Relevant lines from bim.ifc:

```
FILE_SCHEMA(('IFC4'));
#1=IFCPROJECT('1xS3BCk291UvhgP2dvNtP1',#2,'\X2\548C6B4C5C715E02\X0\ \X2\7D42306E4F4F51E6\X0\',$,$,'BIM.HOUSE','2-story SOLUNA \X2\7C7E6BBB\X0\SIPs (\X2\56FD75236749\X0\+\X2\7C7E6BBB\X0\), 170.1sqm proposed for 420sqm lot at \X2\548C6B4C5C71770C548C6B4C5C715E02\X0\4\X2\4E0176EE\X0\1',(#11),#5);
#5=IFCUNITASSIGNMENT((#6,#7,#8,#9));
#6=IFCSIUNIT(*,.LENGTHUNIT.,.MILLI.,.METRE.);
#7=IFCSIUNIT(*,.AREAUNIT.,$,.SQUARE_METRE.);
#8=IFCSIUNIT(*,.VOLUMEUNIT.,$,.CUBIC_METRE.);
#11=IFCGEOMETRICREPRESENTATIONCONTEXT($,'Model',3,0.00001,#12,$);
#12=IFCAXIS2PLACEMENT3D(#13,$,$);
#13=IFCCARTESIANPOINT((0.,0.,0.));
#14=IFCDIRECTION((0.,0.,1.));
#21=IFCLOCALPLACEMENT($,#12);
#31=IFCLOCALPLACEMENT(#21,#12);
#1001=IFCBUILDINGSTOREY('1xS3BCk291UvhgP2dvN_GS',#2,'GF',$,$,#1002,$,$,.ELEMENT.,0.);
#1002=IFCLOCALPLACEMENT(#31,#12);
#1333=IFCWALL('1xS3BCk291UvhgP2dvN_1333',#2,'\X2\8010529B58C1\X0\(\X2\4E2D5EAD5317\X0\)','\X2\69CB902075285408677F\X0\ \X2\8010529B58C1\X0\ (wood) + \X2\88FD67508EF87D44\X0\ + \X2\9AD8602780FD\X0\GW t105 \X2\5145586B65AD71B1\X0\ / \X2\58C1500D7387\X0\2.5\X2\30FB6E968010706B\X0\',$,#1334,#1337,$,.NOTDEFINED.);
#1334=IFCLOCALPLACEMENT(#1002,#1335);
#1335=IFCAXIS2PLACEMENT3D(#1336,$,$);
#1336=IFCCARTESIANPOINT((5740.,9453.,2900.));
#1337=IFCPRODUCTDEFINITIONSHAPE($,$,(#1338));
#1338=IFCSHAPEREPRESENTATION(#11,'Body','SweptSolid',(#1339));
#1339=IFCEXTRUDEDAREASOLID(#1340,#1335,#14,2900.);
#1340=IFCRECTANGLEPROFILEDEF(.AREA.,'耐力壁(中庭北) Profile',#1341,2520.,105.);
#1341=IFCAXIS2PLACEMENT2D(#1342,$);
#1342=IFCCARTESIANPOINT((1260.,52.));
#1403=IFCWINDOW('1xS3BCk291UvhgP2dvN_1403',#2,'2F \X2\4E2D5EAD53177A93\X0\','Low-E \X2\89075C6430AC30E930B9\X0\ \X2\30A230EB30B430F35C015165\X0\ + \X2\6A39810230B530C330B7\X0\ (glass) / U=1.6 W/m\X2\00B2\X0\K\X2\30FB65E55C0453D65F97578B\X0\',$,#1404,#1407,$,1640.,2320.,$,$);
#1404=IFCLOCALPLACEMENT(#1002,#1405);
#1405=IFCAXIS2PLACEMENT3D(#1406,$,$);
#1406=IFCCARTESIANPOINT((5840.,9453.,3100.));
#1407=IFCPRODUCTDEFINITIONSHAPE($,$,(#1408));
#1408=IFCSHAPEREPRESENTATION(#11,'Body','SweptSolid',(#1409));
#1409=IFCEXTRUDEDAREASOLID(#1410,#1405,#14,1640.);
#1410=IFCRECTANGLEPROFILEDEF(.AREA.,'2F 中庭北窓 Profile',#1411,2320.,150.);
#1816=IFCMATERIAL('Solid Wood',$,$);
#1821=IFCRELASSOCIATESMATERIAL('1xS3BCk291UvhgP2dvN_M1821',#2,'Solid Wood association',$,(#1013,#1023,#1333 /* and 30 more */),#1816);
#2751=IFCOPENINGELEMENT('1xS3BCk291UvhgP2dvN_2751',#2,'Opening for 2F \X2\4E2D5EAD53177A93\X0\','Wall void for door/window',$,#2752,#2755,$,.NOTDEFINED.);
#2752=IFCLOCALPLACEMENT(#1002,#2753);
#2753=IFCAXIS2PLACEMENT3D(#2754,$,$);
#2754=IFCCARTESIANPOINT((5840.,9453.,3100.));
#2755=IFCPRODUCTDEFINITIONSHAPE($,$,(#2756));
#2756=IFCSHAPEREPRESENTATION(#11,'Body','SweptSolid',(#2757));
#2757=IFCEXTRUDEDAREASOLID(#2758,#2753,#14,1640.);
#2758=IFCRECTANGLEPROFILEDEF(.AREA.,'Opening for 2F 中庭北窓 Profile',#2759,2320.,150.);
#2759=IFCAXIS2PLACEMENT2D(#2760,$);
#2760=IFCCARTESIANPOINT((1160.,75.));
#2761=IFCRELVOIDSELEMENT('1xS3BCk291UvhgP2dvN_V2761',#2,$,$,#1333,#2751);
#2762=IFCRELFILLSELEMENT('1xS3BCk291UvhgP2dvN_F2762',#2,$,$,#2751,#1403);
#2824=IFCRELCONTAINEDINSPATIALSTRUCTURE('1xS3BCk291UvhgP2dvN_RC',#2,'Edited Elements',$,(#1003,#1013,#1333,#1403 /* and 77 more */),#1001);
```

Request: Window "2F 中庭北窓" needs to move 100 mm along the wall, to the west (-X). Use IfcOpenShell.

```python
import ifcopenshell
import ifcopenshell.api.geometry
import ifcopenshell.util.placement

model = ifcopenshell.open("bim.ifc")

window = model.by_id(1403)
opening = window.FillsVoids[0].RelatingOpeningElement
wall = opening.VoidsElements[0].RelatingBuildingElement

wall_matrix = ifcopenshell.util.placement.get_local_placement(wall.ObjectPlacement)
shift = wall_matrix[:3, 0] * -100.0
before = ifcopenshell.util.placement.get_local_placement(window.ObjectPlacement)[:3, 3].copy()

# The window is not placed relative to its opening, so move both.
for product in (opening, window):
    matrix = ifcopenshell.util.placement.get_local_placement(product.ObjectPlacement)
    matrix[:3, 3] += shift
    ifcopenshell.api.geometry.edit_object_placement(model, product=product, matrix=matrix, is_si=False)

after = ifcopenshell.util.placement.get_local_placement(window.ObjectPlacement)[:3, 3]
print("window moved by", (after - before).round(3) + 0.0)

model.write("bim_v2.ifc")
```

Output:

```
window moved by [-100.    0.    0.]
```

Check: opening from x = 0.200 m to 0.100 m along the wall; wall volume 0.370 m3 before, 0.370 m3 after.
